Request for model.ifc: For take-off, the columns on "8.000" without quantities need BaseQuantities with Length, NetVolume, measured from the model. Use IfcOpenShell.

First a look at what the model holds.

```python
import ifcopenshell
import ifcopenshell.util.element
import ifcopenshell.util.unit

model = ifcopenshell.open("model.ifc")
print(model.schema)
for unit_type in ("LENGTHUNIT", "AREAUNIT", "VOLUMEUNIT"):
    print(unit_type, ifcopenshell.util.unit.calculate_unit_scale(model, unit_type))
storey = next(s for s in model.by_type("IfcBuildingStorey") if s.Name == "8.000")
columns = [e for e in ifcopenshell.util.element.get_decomposition(storey) if e.is_a("IfcColumn")]
for e in sorted(columns, key=lambda e: e.id()):
    print(e.id(), e.is_a(), e.Name, list(ifcopenshell.util.element.get_psets(e, qtos_only=True)), sep=" | ")
```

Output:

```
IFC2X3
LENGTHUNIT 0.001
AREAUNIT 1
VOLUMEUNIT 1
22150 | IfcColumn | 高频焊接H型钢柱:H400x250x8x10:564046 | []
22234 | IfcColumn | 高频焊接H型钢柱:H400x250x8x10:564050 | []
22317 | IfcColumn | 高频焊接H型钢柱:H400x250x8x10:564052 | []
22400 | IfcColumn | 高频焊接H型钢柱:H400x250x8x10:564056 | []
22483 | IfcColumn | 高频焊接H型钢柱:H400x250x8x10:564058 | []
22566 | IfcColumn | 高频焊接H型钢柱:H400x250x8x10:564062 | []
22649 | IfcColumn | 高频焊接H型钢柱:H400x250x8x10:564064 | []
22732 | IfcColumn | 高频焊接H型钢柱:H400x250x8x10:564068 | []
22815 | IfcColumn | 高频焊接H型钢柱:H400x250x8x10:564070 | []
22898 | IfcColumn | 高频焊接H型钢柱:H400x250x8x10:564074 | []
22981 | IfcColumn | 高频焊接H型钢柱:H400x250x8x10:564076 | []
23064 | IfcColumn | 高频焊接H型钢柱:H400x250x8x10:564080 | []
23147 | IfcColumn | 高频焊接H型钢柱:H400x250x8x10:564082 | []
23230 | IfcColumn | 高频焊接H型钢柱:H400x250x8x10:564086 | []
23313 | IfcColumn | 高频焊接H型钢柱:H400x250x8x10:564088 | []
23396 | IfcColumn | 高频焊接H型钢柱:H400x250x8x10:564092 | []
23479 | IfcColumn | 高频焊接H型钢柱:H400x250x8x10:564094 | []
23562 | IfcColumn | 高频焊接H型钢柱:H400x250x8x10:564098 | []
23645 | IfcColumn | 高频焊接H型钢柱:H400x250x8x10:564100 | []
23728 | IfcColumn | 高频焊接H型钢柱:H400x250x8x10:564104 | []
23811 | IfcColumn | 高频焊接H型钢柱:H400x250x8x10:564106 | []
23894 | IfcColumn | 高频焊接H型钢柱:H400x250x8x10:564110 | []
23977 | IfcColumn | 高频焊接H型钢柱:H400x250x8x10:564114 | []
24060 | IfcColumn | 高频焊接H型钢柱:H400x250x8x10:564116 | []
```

```python
import ifcopenshell
import ifcopenshell.api.pset
import ifcopenshell.geom
import ifcopenshell.util.element
import ifcopenshell.util.shape
import ifcopenshell.util.unit

model = ifcopenshell.open("model.ifc")
unit_scale = ifcopenshell.util.unit.calculate_unit_scale(model)
volume_scale = ifcopenshell.util.unit.calculate_unit_scale(model, "VOLUMEUNIT")
settings = ifcopenshell.geom.settings()

storey = next(s for s in model.by_type("IfcBuildingStorey") if s.Name == "8.000")
columns = [e for e in ifcopenshell.util.element.get_decomposition(storey) if e.is_a("IfcColumn")]

for e in sorted(columns, key=lambda e: e.id()):
    if ifcopenshell.util.element.get_psets(e, qtos_only=True, should_inherit=False):
        continue
    # Geometry comes back in metres, in the element's own axes.
    shape = ifcopenshell.geom.create_shape(settings, e)
    values = {
        "Length": ifcopenshell.util.shape.get_z(shape.geometry) / unit_scale,
        "NetVolume": ifcopenshell.util.shape.get_volume(shape.geometry) / volume_scale,
    }
    qto = ifcopenshell.api.pset.add_qto(model, product=e, name="BaseQuantities")
    ifcopenshell.api.pset.edit_qto(model, qto=qto, properties=values)
    print(e.id(), {k: round(v, 3) for k, v in values.items()})

model.write("model_v2.ifc")
```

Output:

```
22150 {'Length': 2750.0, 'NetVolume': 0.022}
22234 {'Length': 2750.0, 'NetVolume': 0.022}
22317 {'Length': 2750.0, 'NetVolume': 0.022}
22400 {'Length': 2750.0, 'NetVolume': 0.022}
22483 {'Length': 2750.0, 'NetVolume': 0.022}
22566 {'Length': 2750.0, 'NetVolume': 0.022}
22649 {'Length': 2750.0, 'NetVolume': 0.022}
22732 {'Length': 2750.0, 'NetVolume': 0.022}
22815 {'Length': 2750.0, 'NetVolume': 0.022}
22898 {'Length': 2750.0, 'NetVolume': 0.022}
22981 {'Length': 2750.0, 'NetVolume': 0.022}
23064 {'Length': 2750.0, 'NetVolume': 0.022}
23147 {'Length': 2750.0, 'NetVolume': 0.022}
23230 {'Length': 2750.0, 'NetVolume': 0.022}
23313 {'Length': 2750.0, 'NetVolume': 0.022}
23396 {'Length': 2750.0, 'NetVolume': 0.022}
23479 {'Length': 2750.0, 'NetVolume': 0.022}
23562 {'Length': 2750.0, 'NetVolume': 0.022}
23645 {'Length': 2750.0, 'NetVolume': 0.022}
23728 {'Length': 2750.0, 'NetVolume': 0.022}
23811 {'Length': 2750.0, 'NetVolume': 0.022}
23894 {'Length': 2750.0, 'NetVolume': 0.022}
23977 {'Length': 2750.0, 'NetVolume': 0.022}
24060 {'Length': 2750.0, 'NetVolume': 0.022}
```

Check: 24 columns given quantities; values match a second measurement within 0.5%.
